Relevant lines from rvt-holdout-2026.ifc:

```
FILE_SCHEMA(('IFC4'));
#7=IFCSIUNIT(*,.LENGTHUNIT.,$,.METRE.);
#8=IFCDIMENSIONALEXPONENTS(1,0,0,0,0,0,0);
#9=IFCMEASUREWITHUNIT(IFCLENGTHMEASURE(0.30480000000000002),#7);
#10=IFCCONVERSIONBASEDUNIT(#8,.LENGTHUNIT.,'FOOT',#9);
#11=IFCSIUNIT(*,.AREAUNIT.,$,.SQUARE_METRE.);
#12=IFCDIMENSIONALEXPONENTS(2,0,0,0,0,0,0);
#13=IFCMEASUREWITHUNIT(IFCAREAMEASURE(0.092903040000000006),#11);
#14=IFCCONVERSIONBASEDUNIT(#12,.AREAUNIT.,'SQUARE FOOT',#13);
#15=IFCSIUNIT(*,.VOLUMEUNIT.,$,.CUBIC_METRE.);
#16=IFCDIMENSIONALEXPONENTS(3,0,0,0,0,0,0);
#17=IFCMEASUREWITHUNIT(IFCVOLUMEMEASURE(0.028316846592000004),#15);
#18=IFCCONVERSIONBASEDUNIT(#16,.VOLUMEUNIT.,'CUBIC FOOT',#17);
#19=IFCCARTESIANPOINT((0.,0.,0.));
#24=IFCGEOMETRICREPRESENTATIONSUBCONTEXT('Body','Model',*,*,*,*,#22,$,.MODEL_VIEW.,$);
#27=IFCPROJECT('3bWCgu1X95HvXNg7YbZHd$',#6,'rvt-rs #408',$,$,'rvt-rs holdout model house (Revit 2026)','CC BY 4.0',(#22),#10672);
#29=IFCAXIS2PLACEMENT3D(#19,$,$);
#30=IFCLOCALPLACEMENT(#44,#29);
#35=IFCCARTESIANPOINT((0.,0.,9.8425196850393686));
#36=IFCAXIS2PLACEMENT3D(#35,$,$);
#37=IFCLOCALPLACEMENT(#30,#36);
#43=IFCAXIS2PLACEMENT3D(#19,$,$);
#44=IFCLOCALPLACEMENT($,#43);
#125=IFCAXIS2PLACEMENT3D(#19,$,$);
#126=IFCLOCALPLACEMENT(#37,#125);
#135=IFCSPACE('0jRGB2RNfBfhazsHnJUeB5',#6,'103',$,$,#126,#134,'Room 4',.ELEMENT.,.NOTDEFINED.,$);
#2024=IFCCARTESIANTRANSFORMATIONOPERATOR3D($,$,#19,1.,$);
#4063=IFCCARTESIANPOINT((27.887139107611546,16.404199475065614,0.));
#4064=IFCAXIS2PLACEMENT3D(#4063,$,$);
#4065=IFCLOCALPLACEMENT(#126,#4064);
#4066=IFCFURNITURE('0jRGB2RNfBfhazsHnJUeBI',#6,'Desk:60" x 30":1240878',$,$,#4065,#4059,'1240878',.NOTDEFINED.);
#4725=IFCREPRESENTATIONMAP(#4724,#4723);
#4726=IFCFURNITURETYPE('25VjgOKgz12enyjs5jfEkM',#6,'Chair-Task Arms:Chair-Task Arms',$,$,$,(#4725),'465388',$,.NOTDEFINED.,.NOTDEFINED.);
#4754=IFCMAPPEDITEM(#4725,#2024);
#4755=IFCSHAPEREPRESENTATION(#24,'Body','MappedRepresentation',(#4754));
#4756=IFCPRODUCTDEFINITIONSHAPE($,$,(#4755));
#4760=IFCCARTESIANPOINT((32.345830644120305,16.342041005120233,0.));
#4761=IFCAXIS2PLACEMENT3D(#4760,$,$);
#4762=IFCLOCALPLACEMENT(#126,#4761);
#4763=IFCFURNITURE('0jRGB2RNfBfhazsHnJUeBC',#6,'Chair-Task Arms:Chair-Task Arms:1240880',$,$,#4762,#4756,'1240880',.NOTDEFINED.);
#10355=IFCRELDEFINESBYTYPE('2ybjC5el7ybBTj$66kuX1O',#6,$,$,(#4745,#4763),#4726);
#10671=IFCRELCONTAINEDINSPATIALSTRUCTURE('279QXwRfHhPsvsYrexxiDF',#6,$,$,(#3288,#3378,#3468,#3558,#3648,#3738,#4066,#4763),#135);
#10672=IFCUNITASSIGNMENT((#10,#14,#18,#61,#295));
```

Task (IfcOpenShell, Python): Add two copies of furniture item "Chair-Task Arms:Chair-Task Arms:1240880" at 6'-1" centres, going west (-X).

```python
import numpy as np
import ifcopenshell
import ifcopenshell.api.geometry
import ifcopenshell.api.root
import ifcopenshell.util.element
import ifcopenshell.util.placement
import ifcopenshell.util.unit

model = ifcopenshell.open("rvt-holdout-2026.ifc")
unit_scale = ifcopenshell.util.unit.calculate_unit_scale(model)


def reuse_history(source, copy):
    """copy_class also copies each property set's owner history, people and application; keep the originals."""
    for rel in copy.IsDefinedBy:
        if rel.is_a("IfcRelDefinesByProperties") and (history := rel.RelatingPropertyDefinition.OwnerHistory):
            rel.RelatingPropertyDefinition.OwnerHistory = source.OwnerHistory
            ifcopenshell.util.element.remove_deep2(model, history)


source = model.by_id(4763)
base = ifcopenshell.util.placement.get_local_placement(source.ObjectPlacement)
step = np.array([-1.0, 0.0, 0.0]) * 73 * 0.0254 / unit_scale

for i in range(1, 3):
    copy = ifcopenshell.api.root.copy_class(model, product=source)
    copy.Representation = ifcopenshell.util.element.copy_deep(
        model, source.Representation, exclude=["IfcGeometricRepresentationContext", "IfcRepresentationMap"]
    )
    copy.Name = "Chair-Task Arms:Chair-Task Arms"
    copy.Tag = None
    reuse_history(source, copy)
    matrix = base.copy()
    matrix[:3, 3] += i * step
    print("added at", matrix[:3, 3].round(3) + 0.0)
    ifcopenshell.api.geometry.edit_object_placement(model, product=copy, matrix=matrix, is_si=False)

model.write("rvt-holdout-2026-out.ifc")
```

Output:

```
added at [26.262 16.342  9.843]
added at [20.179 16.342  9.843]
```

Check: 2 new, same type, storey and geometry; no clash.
